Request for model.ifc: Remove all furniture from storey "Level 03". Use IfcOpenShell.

First a look at what the model holds.

```python
import ifcopenshell
import ifcopenshell.util.element

model = ifcopenshell.open("model.ifc")
print(model.schema)
storey = next(s for s in model.by_type("IfcBuildingStorey") if s.Name == "Level 03")
furniture = [e for e in ifcopenshell.util.element.get_decomposition(storey) if e.is_a("IfcFurnishingElement")]
seen = {}
for e in furniture:
    element_type = ifcopenshell.util.element.get_type(e)
    name = element_type.Name if element_type not in (None, e) else None
    seen[name] = seen.get(name, 0) + 1
for name, count in sorted(seen.items(), key=str):
    print(count, "x", name)
```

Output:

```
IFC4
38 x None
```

```python
import ifcopenshell
import ifcopenshell.api.root
import ifcopenshell.util.element

model = ifcopenshell.open("model.ifc")

storey = next(s for s in model.by_type("IfcBuildingStorey") if s.Name == "Level 03")
furniture = [e for e in ifcopenshell.util.element.get_decomposition(storey) if e.is_a("IfcFurnishingElement")]

for e in furniture:
    ifcopenshell.api.root.remove_product(model, product=e)
print(len(furniture), "removed")

model.write("model_updated.ifc")
```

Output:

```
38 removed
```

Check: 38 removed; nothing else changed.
